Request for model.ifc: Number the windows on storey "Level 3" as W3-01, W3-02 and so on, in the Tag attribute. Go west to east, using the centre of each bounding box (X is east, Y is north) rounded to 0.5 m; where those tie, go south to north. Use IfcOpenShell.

First a look at what the model holds.

```python
import ifcopenshell
import ifcopenshell.util.element
import ifcopenshell.util.placement

model = ifcopenshell.open("model.ifc")
print(model.schema)
storey = next(s for s in model.by_type("IfcBuildingStorey") if s.Name == "Level 3")
windows = [e for e in ifcopenshell.util.element.get_decomposition(storey) if e.is_a("IfcWindow")]
for e in sorted(windows, key=lambda e: e.id()):
    origin = ifcopenshell.util.placement.get_local_placement(e.ObjectPlacement)[:3, 3]
    print(e.id(), e.Tag, e.Name, origin.round(2) + 0.0, sep=" | ")
```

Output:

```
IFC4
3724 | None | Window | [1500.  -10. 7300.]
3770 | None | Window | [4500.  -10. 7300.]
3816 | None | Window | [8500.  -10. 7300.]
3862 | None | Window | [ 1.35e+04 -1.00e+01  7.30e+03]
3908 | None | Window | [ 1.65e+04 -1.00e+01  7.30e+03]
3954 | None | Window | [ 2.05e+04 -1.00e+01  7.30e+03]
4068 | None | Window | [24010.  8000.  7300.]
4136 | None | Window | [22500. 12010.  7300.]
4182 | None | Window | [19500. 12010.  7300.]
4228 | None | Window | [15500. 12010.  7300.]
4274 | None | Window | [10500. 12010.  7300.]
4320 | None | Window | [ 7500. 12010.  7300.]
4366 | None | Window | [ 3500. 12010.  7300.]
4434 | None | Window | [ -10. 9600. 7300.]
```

```python
import ifcopenshell
import ifcopenshell.geom
import ifcopenshell.util.element
import ifcopenshell.util.shape

model = ifcopenshell.open("model.ifc")
settings = ifcopenshell.geom.settings()
settings.set("use-world-coords", True)


def centre(element):
    shape = ifcopenshell.geom.create_shape(settings, element)
    return ifcopenshell.util.shape.get_bbox_centroid(shape.geometry)


storey = next(s for s in model.by_type("IfcBuildingStorey") if s.Name == "Level 3")
windows = [e for e in ifcopenshell.util.element.get_decomposition(storey) if e.is_a("IfcWindow")]

# Insertion points can sit at a corner or the storey origin, so sort by the geometry (in metres).
centres = {e: centre(e) for e in windows}
windows.sort(key=lambda e: (round(centres[e][0] / 0.5), centres[e][1]))

for i, e in enumerate(windows, start=1):
    number = f"W3-{i:02d}"
    e.Tag = number
    print(e.id(), number)

model.write("model_edited.ifc")
```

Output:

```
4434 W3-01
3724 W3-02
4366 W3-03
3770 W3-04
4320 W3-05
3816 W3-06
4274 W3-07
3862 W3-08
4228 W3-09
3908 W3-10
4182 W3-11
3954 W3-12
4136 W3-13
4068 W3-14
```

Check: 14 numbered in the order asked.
